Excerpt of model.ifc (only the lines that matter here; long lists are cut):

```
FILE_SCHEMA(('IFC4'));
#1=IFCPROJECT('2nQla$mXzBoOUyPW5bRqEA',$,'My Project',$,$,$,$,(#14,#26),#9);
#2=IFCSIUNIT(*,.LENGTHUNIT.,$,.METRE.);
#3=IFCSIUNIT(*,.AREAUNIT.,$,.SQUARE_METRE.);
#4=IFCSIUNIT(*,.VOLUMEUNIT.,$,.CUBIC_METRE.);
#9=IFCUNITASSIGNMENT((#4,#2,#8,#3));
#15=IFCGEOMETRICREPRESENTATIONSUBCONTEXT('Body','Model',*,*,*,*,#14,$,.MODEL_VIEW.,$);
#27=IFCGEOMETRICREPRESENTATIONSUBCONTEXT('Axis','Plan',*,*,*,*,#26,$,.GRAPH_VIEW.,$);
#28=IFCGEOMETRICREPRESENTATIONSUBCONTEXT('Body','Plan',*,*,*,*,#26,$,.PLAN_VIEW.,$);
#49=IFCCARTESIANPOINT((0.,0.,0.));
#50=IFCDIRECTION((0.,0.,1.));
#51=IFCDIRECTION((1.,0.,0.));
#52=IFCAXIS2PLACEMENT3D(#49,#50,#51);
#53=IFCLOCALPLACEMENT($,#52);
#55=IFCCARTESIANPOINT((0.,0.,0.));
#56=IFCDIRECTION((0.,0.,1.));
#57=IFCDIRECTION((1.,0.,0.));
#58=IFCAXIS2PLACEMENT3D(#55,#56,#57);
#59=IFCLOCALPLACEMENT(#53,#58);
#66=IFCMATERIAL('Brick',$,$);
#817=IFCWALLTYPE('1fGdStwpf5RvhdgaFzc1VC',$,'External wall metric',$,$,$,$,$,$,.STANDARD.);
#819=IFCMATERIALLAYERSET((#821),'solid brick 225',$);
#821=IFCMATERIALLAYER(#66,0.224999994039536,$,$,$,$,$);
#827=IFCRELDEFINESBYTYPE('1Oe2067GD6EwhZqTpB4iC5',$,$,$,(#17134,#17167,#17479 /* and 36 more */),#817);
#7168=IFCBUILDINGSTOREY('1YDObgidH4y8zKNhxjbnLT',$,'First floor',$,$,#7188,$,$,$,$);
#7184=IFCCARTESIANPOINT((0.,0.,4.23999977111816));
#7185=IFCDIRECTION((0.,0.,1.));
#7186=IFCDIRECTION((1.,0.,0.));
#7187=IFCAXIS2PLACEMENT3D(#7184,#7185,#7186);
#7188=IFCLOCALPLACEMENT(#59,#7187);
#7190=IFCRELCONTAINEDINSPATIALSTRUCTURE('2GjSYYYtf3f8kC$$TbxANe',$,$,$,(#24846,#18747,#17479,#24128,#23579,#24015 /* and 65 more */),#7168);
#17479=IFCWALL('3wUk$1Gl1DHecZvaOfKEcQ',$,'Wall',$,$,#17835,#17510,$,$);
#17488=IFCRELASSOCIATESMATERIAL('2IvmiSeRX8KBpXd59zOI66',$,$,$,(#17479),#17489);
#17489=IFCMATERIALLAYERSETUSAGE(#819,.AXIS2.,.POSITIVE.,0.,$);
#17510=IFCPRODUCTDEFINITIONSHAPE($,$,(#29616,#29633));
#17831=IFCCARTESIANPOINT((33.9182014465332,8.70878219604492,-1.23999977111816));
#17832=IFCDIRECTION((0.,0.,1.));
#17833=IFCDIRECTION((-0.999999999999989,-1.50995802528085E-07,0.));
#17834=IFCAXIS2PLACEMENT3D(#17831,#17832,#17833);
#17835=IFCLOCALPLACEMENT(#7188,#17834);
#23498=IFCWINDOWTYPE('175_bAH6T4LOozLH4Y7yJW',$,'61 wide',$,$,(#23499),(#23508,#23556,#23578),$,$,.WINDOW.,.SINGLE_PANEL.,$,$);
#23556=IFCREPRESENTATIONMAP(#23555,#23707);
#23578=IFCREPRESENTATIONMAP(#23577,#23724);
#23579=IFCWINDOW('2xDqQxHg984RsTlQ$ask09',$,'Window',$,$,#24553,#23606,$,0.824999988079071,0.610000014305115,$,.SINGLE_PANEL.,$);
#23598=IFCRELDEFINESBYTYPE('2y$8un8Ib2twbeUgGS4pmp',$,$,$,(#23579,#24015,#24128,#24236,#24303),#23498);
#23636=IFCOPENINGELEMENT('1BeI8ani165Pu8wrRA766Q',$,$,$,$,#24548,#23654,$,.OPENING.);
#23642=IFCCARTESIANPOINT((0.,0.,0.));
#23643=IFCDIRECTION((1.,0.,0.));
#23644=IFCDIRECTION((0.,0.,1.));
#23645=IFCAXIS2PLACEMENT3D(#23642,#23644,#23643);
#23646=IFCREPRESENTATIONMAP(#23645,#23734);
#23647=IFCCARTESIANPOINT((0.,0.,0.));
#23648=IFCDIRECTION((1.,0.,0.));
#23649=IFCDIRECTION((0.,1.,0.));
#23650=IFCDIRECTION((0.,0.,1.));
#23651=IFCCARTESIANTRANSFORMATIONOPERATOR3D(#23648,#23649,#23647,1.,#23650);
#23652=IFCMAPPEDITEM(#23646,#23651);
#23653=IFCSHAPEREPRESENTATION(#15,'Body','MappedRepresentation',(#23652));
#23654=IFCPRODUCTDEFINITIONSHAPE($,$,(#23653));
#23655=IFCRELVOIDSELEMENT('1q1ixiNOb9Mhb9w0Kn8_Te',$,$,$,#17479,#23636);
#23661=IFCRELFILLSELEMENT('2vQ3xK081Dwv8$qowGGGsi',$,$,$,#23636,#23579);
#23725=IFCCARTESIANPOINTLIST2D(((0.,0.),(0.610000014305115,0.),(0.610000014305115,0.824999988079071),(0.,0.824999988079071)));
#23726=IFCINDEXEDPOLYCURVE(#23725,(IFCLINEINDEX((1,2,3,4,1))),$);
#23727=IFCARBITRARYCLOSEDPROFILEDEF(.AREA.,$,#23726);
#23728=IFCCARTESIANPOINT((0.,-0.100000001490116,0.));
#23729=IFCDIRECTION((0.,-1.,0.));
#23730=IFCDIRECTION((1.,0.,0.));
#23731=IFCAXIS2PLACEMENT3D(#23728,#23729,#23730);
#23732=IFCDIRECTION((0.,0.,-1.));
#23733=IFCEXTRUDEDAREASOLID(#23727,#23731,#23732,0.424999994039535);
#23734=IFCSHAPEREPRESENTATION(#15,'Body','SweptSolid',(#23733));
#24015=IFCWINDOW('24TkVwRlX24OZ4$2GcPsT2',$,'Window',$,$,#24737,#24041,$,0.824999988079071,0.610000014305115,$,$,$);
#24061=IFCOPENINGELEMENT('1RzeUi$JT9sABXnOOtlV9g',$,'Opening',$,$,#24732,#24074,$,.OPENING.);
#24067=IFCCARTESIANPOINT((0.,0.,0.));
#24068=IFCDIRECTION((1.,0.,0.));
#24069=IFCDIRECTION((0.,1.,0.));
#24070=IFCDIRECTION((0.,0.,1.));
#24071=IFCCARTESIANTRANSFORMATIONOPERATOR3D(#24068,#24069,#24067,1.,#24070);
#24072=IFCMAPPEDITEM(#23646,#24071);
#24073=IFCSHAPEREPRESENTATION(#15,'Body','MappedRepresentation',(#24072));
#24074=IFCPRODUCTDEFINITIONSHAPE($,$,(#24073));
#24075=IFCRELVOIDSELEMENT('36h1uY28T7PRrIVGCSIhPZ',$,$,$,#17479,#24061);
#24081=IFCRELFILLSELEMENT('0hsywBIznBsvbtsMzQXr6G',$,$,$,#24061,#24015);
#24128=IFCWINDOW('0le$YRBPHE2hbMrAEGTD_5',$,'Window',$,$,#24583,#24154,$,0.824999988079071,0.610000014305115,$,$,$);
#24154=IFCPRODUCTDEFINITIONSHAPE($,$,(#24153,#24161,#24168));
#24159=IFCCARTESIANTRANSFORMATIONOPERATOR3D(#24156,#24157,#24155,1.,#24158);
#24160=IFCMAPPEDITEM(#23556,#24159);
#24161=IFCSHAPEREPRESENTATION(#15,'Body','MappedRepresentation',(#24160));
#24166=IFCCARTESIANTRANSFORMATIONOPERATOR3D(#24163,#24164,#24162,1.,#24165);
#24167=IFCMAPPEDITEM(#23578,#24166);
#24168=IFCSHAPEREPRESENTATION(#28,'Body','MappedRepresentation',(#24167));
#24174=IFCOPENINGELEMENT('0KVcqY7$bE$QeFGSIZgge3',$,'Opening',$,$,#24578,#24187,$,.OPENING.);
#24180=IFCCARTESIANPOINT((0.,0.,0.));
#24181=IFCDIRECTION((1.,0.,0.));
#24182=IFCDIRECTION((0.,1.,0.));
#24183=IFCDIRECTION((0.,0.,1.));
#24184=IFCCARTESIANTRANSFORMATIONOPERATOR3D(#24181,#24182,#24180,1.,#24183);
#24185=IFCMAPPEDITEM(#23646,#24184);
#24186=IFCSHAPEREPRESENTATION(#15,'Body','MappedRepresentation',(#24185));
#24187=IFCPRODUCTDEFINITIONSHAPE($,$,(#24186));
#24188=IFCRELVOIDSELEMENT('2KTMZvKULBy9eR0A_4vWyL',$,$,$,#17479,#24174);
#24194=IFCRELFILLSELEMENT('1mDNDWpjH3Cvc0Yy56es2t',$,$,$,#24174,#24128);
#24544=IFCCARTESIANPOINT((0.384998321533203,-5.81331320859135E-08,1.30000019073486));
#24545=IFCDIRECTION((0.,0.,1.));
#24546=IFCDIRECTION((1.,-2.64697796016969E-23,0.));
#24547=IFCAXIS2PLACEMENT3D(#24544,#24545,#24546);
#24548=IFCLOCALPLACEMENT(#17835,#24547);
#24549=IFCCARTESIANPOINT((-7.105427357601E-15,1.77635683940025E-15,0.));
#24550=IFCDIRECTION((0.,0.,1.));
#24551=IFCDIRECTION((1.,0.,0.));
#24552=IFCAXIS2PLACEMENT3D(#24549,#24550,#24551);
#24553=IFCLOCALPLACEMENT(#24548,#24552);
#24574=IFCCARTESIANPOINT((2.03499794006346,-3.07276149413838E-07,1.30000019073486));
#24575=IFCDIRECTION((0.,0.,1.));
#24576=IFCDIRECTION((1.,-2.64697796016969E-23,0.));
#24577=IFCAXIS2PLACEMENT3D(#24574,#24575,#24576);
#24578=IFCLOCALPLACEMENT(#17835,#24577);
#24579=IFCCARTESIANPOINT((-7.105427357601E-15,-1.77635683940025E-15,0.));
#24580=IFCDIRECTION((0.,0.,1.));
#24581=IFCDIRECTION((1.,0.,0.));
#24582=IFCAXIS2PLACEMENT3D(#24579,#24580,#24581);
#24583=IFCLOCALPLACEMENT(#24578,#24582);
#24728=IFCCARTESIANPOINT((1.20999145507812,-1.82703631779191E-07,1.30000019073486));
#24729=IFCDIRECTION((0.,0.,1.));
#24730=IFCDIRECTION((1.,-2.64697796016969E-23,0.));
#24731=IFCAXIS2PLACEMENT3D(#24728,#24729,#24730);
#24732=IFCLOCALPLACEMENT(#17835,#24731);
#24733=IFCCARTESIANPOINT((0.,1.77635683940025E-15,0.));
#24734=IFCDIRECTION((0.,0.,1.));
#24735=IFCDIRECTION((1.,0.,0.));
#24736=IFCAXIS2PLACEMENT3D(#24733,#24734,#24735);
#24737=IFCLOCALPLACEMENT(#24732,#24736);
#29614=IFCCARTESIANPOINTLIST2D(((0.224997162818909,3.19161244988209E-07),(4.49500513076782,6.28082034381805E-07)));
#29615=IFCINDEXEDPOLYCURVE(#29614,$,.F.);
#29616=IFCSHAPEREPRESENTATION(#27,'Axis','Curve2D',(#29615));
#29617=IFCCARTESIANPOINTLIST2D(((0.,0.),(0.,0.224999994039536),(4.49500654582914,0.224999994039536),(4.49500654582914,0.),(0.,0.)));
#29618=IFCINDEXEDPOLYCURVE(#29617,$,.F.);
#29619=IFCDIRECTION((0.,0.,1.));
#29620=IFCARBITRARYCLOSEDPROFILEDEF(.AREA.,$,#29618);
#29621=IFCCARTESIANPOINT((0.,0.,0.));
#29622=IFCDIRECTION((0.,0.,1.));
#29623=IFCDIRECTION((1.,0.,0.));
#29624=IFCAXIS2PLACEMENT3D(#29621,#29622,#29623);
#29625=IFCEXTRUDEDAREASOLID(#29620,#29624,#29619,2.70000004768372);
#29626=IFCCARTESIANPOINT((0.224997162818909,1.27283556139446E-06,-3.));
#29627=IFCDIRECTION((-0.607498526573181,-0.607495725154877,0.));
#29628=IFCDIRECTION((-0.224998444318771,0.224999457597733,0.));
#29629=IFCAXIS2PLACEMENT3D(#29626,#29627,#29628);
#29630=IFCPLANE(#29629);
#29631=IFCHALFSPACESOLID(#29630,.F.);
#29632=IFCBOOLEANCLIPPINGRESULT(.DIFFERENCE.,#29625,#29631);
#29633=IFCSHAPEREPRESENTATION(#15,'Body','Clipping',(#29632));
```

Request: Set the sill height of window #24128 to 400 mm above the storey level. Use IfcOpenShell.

```python
import numpy as np
import ifcopenshell
import ifcopenshell.api.geometry
import ifcopenshell.geom
import ifcopenshell.util.element
import ifcopenshell.util.placement
import ifcopenshell.util.shape
import ifcopenshell.util.unit

model = ifcopenshell.open("model.ifc")
unit_scale = ifcopenshell.util.unit.calculate_unit_scale(model)

window = model.by_guid("0le$YRBPHE2hbMrAEGTD_5")
opening = window.FillsVoids[0].RelatingOpeningElement
storey = ifcopenshell.util.element.get_container(window, ifc_class="IfcBuildingStorey")
level = ifcopenshell.util.placement.get_local_placement(storey.ObjectPlacement)[2, 3]

# The opening's origin need not be at the sill, so measure its lowest point.
shape = ifcopenshell.geom.create_shape(ifcopenshell.geom.settings(), opening)
bottom = ifcopenshell.util.shape.get_shape_bottom_elevation(shape, shape.geometry) / unit_scale
dz = level + 0.4 / unit_scale - bottom

shift = np.array([0.0, 0.0, dz])
# The window is placed relative to its opening, so it follows when the opening moves.
matrix = ifcopenshell.util.placement.get_local_placement(opening.ObjectPlacement)
matrix[:3, 3] += shift
ifcopenshell.api.geometry.edit_object_placement(
    model, product=opening, matrix=matrix, is_si=False, should_transform_children=True
)

print(f"moved by {dz * unit_scale:+.3f} m")

model.write("model-out.ifc")
```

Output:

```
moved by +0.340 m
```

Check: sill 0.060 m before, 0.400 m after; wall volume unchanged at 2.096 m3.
